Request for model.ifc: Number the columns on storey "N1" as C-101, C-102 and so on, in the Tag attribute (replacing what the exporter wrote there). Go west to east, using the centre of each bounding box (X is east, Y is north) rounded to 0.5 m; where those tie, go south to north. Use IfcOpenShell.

First a look at what the model holds.

```python
import ifcopenshell
import ifcopenshell.util.element
import ifcopenshell.util.placement

model = ifcopenshell.open("model.ifc")
print(model.schema)
storey = next(s for s in model.by_type("IfcBuildingStorey") if s.Name == "N1")
columns = [e for e in ifcopenshell.util.element.get_decomposition(storey) if e.is_a("IfcColumn")]
for e in sorted(columns, key=lambda e: e.id()):
    origin = ifcopenshell.util.placement.get_local_placement(e.ObjectPlacement)[:3, 3]
    print(e.id(), e.Tag, e.Name, origin.round(2) + 0.0, sep=" | ")
```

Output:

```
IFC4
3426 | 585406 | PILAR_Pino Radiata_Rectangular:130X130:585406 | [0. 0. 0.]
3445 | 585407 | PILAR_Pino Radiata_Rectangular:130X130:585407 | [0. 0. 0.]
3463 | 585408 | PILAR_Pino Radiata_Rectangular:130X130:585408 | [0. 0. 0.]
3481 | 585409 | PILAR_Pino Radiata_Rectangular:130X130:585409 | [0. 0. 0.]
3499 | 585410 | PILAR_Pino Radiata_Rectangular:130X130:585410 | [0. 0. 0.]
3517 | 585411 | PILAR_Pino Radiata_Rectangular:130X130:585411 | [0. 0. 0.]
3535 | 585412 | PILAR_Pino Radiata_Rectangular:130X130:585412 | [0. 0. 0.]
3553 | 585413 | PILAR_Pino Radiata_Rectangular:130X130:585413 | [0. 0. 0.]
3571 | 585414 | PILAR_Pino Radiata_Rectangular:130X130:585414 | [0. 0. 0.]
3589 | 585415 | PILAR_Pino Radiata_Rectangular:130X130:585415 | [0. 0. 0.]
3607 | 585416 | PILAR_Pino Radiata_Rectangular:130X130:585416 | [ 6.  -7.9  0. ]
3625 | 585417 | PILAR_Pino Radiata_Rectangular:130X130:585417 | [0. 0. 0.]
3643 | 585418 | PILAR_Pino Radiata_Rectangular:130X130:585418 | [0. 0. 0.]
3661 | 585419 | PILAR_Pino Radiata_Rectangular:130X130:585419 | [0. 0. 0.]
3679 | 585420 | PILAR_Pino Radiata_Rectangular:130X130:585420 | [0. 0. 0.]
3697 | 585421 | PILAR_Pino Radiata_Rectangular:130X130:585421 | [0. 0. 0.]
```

```python
import ifcopenshell
import ifcopenshell.geom
import ifcopenshell.util.element
import ifcopenshell.util.shape

model = ifcopenshell.open("model.ifc")
settings = ifcopenshell.geom.settings()
settings.set("use-world-coords", True)


def centre(element):
    shape = ifcopenshell.geom.create_shape(settings, element)
    return ifcopenshell.util.shape.get_bbox_centroid(shape.geometry)


storey = next(s for s in model.by_type("IfcBuildingStorey") if s.Name == "N1")
columns = [e for e in ifcopenshell.util.element.get_decomposition(storey) if e.is_a("IfcColumn")]

# Insertion points can sit at a corner or the storey origin, so sort by the geometry (in metres).
centres = {e: centre(e) for e in columns}
columns.sort(key=lambda e: (round(centres[e][0] / 0.5), centres[e][1]))

for i, e in enumerate(columns, start=1):
    number = f"C-1{i:02d}"
    e.Tag = number
    print(e.id(), number)

model.write("model_v2.ifc")
```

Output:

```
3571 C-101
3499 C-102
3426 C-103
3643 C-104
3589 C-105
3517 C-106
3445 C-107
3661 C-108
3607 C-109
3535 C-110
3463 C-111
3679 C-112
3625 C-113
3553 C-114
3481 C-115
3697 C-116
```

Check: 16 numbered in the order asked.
